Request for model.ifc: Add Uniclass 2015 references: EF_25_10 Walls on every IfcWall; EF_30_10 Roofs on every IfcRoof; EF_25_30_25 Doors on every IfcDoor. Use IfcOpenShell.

First a look at what the model holds.

```python
import ifcopenshell

model = ifcopenshell.open("model.ifc")
print(model.schema)
print("classifications:", [c.Name for c in model.by_type("IfcClassification")])
for ifc_class in ("IfcDoor", "IfcRoof", "IfcStair", "IfcWall", "IfcWindow"):
    print(ifc_class, len(model.by_type(ifc_class)))
```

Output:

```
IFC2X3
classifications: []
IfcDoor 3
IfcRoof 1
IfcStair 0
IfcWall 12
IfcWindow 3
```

```python
import ifcopenshell
import ifcopenshell.api.classification

model = ifcopenshell.open("model.ifc")

# IFC2X3 requires Source and Edition and has no link from the project to the system.
system = model.create_entity("IfcClassification", Source="NBS", Edition="2015", Name="Uniclass 2015")

codes = {
    "IfcWall": ("EF_25_10", "Walls"),
    "IfcRoof": ("EF_30_10", "Roofs"),
    "IfcDoor": ("EF_25_30_25", "Doors"),
}
for ifc_class, (code, name) in codes.items():
    products = model.by_type(ifc_class)
    ifcopenshell.api.classification.add_reference(
        model, products=products, classification=system, identification=code, name=name
    )
    print(code, len(products))

model.write("model-out.ifc")
```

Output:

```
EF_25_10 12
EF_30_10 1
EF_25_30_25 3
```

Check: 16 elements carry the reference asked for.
